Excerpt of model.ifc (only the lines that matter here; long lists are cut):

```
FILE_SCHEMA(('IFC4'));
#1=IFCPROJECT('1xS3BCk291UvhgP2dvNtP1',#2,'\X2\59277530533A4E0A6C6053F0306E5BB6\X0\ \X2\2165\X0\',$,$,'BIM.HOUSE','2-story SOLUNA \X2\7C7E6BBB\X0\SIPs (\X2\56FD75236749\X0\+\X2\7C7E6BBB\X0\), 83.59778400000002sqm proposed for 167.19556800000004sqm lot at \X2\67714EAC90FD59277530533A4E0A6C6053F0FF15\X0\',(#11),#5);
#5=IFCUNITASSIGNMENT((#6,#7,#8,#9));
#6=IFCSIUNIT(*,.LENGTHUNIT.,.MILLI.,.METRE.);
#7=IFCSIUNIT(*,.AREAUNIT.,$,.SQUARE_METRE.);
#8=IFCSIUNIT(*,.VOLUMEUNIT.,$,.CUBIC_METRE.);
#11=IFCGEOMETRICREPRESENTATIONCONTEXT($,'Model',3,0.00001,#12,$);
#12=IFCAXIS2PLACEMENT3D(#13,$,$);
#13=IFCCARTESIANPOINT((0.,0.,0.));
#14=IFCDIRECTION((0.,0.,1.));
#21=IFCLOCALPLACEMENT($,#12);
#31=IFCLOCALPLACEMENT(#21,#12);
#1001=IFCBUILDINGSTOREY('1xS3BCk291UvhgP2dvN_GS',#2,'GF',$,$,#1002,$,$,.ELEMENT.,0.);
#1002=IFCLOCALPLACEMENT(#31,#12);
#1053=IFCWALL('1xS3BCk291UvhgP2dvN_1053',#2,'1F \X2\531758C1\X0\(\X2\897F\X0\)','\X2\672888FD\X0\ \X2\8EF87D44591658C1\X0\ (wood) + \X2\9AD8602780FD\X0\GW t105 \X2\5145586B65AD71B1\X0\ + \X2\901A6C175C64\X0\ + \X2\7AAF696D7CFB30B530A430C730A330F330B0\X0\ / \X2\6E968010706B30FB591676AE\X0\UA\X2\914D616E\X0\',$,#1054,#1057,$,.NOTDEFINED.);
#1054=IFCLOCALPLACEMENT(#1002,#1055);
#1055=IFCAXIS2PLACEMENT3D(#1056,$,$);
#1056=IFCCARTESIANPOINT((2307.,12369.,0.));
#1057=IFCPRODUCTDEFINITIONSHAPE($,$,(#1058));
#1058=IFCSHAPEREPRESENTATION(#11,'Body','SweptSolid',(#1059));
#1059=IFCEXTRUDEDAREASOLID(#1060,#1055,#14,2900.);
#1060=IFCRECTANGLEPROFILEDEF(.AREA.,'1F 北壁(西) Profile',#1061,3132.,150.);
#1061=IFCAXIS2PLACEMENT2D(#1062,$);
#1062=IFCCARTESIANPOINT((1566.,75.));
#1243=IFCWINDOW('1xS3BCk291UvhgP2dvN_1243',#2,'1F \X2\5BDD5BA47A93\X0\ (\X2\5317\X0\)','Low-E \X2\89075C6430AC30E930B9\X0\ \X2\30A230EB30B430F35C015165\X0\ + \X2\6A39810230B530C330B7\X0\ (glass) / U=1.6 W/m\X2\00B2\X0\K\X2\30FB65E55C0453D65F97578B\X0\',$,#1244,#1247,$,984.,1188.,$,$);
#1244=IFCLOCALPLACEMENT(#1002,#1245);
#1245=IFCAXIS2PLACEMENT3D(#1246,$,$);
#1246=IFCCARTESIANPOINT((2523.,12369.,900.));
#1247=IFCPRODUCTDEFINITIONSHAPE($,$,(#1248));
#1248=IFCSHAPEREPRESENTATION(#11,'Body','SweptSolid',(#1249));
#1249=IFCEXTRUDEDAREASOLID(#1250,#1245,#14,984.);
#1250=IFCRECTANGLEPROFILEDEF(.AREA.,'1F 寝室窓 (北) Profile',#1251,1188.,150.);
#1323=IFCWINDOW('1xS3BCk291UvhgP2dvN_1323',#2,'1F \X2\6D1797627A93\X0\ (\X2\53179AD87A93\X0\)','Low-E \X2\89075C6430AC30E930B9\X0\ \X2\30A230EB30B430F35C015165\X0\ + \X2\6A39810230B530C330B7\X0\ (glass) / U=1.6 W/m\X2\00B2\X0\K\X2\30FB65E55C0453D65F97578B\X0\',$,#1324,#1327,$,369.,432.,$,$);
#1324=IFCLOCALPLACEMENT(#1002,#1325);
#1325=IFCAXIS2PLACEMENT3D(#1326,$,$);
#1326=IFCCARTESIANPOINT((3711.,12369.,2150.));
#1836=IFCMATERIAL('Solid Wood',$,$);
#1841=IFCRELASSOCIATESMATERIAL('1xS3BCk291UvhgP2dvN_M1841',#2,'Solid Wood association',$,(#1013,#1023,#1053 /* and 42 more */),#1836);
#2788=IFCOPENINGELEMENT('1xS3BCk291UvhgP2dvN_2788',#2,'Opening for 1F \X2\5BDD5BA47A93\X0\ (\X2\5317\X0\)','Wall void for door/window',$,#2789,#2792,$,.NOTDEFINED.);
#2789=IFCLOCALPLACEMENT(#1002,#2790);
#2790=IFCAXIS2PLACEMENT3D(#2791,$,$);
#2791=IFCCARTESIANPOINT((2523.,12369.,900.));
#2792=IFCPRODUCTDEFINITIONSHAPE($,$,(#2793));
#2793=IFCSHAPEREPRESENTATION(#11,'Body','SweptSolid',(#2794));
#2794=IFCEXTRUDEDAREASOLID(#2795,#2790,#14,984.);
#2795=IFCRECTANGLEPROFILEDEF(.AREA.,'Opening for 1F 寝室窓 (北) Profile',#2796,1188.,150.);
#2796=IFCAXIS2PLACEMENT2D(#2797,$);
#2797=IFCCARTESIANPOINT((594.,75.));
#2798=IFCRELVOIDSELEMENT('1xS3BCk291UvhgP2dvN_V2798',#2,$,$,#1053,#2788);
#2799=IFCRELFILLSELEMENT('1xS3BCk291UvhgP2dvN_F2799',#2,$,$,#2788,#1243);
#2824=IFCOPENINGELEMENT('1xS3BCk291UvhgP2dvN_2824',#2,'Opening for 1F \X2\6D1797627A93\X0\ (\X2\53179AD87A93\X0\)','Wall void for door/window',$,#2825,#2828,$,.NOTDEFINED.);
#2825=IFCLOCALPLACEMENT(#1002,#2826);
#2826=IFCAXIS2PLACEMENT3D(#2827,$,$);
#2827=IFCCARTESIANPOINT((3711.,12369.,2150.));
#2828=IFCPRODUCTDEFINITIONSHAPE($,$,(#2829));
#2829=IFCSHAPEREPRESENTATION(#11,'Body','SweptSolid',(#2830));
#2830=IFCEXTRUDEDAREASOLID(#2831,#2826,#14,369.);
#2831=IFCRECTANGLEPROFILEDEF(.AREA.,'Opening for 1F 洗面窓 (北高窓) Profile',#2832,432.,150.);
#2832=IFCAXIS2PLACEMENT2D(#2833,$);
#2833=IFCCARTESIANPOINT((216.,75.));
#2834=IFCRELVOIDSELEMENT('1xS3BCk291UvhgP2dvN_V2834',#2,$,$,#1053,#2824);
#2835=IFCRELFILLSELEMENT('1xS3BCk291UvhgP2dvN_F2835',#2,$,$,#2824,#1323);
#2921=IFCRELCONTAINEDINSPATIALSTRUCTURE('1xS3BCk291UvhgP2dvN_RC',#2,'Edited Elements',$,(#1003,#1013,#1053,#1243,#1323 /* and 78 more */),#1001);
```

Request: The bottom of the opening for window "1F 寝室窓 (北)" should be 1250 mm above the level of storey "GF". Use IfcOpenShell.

```python
import numpy as np
import ifcopenshell
import ifcopenshell.api.geometry
import ifcopenshell.geom
import ifcopenshell.util.element
import ifcopenshell.util.placement
import ifcopenshell.util.shape
import ifcopenshell.util.unit

model = ifcopenshell.open("model.ifc")
unit_scale = ifcopenshell.util.unit.calculate_unit_scale(model)

window = model.by_guid("1xS3BCk291UvhgP2dvN_1243")
opening = window.FillsVoids[0].RelatingOpeningElement
storey = ifcopenshell.util.element.get_container(window, ifc_class="IfcBuildingStorey")
level = ifcopenshell.util.placement.get_local_placement(storey.ObjectPlacement)[2, 3]

# The opening's origin need not be at the sill, so measure its lowest point.
shape = ifcopenshell.geom.create_shape(ifcopenshell.geom.settings(), opening)
bottom = ifcopenshell.util.shape.get_shape_bottom_elevation(shape, shape.geometry) / unit_scale
dz = level + 1.25 / unit_scale - bottom

shift = np.array([0.0, 0.0, dz])
# The window is not placed relative to its opening, so move both.
for product in (opening, window):
    matrix = ifcopenshell.util.placement.get_local_placement(product.ObjectPlacement)
    matrix[:3, 3] += shift
    ifcopenshell.api.geometry.edit_object_placement(model, product=product, matrix=matrix, is_si=False)

print(f"moved by {dz * unit_scale:+.3f} m")

model.write("model_rev.ifc")
```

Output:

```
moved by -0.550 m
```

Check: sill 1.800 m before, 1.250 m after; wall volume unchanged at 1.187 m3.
